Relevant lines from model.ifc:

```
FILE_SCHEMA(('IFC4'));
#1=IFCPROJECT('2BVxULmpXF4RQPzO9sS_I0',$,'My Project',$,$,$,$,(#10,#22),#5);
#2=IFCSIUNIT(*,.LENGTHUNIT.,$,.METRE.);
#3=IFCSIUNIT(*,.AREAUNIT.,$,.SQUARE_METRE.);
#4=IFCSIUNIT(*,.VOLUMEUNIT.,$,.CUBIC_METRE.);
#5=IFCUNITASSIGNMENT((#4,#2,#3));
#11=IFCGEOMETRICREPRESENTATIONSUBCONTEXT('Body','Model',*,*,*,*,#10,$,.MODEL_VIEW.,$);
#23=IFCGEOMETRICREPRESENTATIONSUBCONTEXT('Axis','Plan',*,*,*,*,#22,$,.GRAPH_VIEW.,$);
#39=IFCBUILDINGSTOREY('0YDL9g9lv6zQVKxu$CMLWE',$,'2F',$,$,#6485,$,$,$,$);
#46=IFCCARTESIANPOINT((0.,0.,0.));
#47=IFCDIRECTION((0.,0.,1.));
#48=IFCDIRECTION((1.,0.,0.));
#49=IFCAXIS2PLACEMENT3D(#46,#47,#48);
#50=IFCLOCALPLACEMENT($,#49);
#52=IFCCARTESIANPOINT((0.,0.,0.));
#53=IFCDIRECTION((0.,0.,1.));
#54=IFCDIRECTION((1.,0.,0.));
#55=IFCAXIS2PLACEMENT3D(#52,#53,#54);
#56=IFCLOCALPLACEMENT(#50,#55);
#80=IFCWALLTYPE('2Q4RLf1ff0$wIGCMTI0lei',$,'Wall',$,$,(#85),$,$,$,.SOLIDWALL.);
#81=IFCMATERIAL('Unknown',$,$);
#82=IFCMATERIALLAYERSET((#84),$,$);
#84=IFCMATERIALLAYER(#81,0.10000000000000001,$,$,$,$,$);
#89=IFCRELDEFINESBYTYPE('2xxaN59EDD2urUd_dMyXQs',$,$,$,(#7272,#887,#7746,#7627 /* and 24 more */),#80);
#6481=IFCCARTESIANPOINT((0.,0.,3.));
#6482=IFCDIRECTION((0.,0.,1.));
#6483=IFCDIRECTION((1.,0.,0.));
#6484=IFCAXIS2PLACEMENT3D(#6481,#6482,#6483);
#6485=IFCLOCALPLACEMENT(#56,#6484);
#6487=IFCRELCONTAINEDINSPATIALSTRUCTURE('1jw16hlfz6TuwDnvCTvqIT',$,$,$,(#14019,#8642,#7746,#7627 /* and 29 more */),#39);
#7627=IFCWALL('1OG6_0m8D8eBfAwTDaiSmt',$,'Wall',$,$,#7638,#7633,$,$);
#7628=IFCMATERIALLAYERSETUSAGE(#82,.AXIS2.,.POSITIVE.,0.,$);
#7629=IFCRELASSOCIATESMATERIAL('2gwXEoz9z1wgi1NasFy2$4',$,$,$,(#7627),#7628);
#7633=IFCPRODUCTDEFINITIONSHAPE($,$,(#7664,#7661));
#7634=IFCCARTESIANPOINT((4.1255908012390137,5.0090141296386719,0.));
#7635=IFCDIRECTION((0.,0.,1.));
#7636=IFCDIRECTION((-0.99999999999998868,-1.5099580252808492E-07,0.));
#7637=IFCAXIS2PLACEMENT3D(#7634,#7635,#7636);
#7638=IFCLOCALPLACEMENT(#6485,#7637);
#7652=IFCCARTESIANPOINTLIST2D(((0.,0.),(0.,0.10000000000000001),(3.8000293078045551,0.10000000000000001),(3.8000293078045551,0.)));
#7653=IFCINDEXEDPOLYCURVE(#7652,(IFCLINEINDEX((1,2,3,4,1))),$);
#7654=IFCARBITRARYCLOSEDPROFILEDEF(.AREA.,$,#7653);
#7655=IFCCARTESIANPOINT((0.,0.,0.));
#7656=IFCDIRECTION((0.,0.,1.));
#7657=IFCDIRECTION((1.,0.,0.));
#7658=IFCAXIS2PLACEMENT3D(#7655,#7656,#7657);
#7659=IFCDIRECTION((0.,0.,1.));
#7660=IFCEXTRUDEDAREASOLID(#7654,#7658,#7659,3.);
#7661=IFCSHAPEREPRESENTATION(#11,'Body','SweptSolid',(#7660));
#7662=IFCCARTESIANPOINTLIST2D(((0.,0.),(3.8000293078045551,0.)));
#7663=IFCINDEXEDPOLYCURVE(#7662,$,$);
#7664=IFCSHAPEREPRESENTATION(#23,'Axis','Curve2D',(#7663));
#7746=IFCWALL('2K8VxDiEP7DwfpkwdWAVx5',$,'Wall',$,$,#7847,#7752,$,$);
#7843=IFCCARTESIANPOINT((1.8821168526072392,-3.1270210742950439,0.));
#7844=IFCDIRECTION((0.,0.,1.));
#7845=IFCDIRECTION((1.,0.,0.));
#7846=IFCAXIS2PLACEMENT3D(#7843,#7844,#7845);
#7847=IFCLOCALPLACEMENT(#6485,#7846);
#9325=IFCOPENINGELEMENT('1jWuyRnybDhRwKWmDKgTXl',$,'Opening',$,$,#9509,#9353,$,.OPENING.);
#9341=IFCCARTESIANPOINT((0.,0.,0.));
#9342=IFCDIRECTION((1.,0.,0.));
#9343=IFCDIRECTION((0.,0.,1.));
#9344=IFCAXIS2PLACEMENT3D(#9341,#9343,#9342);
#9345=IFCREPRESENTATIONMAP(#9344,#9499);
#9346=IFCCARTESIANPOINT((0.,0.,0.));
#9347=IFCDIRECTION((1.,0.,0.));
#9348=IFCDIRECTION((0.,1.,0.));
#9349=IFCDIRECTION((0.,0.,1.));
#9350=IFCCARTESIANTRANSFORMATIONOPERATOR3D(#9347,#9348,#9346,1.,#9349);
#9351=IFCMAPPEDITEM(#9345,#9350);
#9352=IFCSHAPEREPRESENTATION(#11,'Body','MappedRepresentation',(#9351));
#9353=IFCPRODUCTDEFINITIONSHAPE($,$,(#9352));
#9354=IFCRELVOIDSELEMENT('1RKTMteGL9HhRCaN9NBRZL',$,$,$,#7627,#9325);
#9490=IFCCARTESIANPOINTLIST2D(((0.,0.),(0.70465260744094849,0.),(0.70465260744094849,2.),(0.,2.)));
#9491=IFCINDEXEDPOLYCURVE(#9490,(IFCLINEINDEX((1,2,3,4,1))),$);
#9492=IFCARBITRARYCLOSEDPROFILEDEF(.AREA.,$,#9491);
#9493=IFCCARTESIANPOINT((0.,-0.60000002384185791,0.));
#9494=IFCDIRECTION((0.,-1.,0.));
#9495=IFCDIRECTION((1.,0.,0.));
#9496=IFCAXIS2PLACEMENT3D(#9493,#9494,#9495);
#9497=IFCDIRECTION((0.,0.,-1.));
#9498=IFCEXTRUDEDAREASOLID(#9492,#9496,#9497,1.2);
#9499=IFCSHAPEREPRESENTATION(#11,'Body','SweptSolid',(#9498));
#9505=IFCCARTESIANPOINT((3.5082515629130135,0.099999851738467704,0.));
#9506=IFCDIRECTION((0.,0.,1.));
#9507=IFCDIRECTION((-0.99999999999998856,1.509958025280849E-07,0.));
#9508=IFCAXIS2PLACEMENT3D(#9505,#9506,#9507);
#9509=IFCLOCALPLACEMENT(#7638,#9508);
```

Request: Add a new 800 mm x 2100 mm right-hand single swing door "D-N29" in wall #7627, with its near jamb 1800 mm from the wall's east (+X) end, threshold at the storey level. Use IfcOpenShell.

```python
import numpy as np
import ifcopenshell
import ifcopenshell.api.feature
import ifcopenshell.api.geometry
import ifcopenshell.api.root
import ifcopenshell.api.spatial
import ifcopenshell.geom
import ifcopenshell.util.element
import ifcopenshell.util.placement
import ifcopenshell.util.representation
import ifcopenshell.util.shape
import ifcopenshell.util.unit

model = ifcopenshell.open("model.ifc")
unit_scale = ifcopenshell.util.unit.calculate_unit_scale(model)
settings = ifcopenshell.geom.settings()


def volume(element):
    """Net volume in cubic metres, openings subtracted."""
    shape = ifcopenshell.geom.create_shape(settings, element)
    return ifcopenshell.util.shape.get_volume(shape.geometry)


wall = model.by_guid("1OG6_0m8D8eBfAwTDaiSmt")
storey = ifcopenshell.util.element.get_container(wall, ifc_class="IfcBuildingStorey")
context = ifcopenshell.util.representation.get_context(model, "Model", "Body", "MODEL_VIEW")
before = volume(wall)

width, height, from_end, sill = 0.8, 2.1, 1.8, 0.0  # metres

# The wall runs along its own X axis, and the end named is its -X end.
wall_shape = ifcopenshell.geom.create_shape(settings, wall)
x, y, z = ifcopenshell.util.shape.get_vertices(wall_shape.geometry).T
start = x.min() + from_end
face, thickness = float(y.min()), float(y.max() - y.min())
wall_matrix = ifcopenshell.util.placement.get_local_placement(wall.ObjectPlacement)
level = ifcopenshell.util.placement.get_local_placement(storey.ObjectPlacement)[2, 3]


def in_wall(x, y):
    """Placement at x, y metres in the wall's axes, at sill height."""
    matrix = wall_matrix.copy()
    matrix[:, 3] = wall_matrix @ np.array([x / unit_scale, y / unit_scale, 0.0, 1.0])
    matrix[2, 3] = level + sill / unit_scale
    return matrix


# Opening: a box that overshoots both wall faces by 50 mm.
opening = ifcopenshell.api.root.create_entity(model, ifc_class="IfcOpeningElement", predefined_type="OPENING")
box = ifcopenshell.api.geometry.add_wall_representation(
    model, context=context, length=width, height=height, thickness=thickness + 0.1
)
ifcopenshell.api.geometry.assign_representation(model, product=opening, representation=box)
ifcopenshell.api.geometry.edit_object_placement(model, product=opening, matrix=in_wall(start, face - 0.05), is_si=False)
ifcopenshell.api.feature.add_feature(model, feature=opening, element=wall)

door = ifcopenshell.api.root.create_entity(model, ifc_class="IfcDoor", name="D-N29", predefined_type="DOOR")
door.OverallWidth, door.OverallHeight = width / unit_scale, height / unit_scale
door.OperationType = "SINGLE_SWING_RIGHT"
body = ifcopenshell.api.geometry.add_door_representation(
    model,
    context=context,
    overall_width=door.OverallWidth,
    overall_height=door.OverallHeight,
    operation_type="SINGLE_SWING_RIGHT",
    lining_properties={"LiningDepth": thickness / unit_scale, "ThresholdDepth": thickness / unit_scale},
)
ifcopenshell.api.geometry.assign_representation(model, product=door, representation=body)
ifcopenshell.api.spatial.assign_container(model, products=[door], relating_structure=storey)
ifcopenshell.api.feature.add_filling(model, opening=opening, element=door)

# The lining spans the wall, so the door starts at the wall face.
ifcopenshell.api.geometry.edit_object_placement(model, product=door, matrix=in_wall(start, face), is_si=False)

after = volume(wall)

print(f"wall volume {before:.3f} -> {after:.3f} m3")

model.write("model_v2.ifc")
```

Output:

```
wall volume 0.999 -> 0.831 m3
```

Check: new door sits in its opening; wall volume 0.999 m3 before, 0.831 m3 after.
